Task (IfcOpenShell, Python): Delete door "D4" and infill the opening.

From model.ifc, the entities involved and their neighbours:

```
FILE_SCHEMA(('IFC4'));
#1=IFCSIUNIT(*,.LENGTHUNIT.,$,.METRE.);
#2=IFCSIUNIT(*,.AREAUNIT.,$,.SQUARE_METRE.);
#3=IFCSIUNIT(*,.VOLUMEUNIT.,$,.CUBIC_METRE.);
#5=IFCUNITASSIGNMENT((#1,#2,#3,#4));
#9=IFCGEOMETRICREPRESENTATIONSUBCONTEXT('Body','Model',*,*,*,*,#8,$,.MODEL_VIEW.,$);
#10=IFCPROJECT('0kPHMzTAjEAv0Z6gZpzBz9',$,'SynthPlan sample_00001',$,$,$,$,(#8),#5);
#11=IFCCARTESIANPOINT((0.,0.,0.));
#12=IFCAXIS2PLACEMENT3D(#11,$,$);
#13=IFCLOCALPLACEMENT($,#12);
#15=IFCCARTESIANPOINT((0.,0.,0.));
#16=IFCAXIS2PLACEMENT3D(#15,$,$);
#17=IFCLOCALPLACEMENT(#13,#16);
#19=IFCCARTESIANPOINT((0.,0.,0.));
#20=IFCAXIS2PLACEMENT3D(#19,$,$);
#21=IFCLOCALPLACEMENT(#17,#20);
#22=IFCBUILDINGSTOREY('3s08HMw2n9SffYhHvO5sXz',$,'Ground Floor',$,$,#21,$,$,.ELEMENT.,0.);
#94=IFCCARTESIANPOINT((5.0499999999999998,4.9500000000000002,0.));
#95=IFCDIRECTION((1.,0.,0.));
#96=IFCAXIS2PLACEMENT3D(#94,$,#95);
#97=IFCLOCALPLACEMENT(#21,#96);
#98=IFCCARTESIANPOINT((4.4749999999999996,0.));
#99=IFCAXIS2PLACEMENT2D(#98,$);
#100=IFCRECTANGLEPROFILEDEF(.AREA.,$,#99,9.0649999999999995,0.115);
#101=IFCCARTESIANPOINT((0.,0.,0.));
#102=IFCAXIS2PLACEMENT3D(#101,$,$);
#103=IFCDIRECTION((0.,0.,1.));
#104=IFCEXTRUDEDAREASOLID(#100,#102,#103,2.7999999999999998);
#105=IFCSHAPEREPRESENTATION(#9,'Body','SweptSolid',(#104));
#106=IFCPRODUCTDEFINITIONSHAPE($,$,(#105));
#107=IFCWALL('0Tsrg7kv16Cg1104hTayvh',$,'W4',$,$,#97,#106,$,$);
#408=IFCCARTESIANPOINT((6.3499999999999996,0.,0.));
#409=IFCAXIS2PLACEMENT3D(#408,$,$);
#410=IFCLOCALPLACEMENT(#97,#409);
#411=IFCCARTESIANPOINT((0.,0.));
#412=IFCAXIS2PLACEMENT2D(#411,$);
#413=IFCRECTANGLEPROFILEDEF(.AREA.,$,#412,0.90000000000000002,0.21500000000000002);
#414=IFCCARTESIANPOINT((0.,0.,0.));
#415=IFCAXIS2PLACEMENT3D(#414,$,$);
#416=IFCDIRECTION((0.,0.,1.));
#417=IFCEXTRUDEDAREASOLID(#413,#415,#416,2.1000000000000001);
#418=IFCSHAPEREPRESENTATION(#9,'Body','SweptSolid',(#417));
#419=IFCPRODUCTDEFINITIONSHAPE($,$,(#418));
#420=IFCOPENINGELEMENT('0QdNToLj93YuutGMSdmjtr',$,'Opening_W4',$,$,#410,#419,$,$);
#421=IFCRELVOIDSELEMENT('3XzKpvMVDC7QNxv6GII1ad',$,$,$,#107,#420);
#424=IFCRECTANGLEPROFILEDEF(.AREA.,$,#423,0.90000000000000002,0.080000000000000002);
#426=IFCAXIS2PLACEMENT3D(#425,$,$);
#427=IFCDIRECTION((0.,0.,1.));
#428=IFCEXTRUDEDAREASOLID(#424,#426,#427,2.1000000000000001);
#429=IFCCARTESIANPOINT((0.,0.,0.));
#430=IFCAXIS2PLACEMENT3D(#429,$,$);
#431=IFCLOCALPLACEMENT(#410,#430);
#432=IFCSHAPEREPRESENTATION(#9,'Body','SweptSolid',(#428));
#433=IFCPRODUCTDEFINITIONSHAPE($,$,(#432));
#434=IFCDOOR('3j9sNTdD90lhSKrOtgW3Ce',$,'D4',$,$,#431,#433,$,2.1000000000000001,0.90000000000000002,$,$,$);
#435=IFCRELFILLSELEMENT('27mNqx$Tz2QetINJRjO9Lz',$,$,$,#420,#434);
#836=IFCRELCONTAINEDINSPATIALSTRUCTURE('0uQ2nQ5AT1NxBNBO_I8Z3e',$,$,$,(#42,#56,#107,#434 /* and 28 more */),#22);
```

```python
import ifcopenshell
import ifcopenshell.api.feature
import ifcopenshell.api.root
import ifcopenshell.geom
import ifcopenshell.util.shape

model = ifcopenshell.open("model.ifc")
settings = ifcopenshell.geom.settings()


def volume(element):
    """Net volume in cubic metres, openings subtracted."""
    shape = ifcopenshell.geom.create_shape(settings, element)
    return ifcopenshell.util.shape.get_volume(shape.geometry)


door = model.by_guid("3j9sNTdD90lhSKrOtgW3Ce")
opening = door.FillsVoids[0].RelatingOpeningElement
wall = opening.VoidsElements[0].RelatingBuildingElement
before = volume(wall)

ifcopenshell.api.root.remove_product(model, product=door)
ifcopenshell.api.feature.remove_feature(model, feature=opening)

after = volume(wall)

print(f"wall volume {before:.3f} -> {after:.3f} m3")

model.write("model_edited.ifc")
```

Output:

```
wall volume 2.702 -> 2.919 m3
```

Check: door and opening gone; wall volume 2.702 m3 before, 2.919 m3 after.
